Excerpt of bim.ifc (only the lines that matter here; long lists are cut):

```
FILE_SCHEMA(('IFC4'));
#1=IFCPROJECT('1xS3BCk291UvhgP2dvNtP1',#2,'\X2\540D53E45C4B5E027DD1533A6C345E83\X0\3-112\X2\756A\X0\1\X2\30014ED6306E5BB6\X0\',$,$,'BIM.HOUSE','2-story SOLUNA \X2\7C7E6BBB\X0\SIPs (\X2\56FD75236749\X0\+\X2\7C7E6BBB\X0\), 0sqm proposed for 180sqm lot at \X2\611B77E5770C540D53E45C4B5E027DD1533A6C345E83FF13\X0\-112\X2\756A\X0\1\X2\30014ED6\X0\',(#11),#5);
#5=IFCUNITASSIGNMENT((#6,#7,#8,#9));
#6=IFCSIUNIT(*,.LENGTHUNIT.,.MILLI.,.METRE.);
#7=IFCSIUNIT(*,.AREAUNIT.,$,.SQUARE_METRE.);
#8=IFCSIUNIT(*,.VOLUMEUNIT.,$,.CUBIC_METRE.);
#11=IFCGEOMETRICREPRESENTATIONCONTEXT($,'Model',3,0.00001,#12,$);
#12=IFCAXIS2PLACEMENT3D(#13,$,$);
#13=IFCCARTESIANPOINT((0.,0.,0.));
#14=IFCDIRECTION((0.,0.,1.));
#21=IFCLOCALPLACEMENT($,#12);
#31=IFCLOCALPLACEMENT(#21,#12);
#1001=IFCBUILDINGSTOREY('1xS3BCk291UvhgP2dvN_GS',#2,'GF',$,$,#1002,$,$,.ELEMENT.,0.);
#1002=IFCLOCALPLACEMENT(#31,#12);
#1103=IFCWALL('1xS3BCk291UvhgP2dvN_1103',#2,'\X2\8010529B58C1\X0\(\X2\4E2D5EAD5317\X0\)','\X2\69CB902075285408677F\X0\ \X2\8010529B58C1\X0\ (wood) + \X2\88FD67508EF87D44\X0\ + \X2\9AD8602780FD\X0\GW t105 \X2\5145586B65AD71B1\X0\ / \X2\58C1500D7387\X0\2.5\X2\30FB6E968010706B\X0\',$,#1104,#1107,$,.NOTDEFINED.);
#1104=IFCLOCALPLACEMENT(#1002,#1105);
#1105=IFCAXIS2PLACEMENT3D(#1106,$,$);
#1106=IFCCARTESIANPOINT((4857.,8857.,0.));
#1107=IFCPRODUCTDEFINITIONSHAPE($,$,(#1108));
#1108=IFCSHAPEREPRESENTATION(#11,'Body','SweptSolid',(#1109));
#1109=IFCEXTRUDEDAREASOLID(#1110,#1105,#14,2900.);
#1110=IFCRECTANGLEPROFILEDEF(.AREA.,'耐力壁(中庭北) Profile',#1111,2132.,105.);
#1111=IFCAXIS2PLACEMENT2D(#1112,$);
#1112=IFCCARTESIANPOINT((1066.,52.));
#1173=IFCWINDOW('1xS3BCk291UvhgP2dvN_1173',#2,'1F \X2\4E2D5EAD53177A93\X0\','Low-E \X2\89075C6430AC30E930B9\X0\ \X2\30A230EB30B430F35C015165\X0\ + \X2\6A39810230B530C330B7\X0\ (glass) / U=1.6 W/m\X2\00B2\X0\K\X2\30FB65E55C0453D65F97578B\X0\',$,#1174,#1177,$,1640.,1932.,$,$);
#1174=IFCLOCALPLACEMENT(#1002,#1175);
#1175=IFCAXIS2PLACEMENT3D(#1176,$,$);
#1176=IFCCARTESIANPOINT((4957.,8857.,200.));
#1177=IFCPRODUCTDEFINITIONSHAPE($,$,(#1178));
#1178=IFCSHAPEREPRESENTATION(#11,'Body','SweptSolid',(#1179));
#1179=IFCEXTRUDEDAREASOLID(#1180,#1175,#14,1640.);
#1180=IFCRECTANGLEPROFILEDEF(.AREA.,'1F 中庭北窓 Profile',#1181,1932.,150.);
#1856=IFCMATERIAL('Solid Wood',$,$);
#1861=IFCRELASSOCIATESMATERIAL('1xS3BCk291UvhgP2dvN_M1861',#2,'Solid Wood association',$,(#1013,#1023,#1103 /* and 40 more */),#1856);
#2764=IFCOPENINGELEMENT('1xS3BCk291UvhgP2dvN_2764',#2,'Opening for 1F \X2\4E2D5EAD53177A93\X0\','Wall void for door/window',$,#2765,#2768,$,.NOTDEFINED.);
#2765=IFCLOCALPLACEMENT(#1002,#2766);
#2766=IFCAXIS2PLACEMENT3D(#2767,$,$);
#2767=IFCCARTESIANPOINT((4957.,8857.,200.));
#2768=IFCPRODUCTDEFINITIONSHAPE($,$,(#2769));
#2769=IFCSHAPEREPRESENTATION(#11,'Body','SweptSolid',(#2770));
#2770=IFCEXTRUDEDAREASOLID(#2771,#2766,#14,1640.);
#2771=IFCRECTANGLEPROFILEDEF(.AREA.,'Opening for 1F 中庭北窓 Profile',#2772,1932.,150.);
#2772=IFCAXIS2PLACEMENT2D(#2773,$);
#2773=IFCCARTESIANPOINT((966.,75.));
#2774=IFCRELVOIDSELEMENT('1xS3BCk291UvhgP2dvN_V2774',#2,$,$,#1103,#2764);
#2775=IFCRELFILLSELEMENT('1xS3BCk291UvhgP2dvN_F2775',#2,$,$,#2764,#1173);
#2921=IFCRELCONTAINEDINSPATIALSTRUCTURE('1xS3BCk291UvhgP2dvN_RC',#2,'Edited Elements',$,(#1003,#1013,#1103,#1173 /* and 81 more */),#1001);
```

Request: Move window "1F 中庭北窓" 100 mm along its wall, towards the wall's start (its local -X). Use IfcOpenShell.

```python
import ifcopenshell
import ifcopenshell.api.geometry
import ifcopenshell.util.placement
import ifcopenshell.util.unit

model = ifcopenshell.open("bim.ifc")
unit_scale = ifcopenshell.util.unit.calculate_unit_scale(model)

window = model.by_guid("1xS3BCk291UvhgP2dvN_1173")
opening = window.FillsVoids[0].RelatingOpeningElement
wall = opening.VoidsElements[0].RelatingBuildingElement

wall_matrix = ifcopenshell.util.placement.get_local_placement(wall.ObjectPlacement)
shift = wall_matrix[:3, 0] * -0.1 / unit_scale
before = ifcopenshell.util.placement.get_local_placement(window.ObjectPlacement)[:3, 3].copy()

# The window is not placed relative to its opening, so move both.
for product in (opening, window):
    matrix = ifcopenshell.util.placement.get_local_placement(product.ObjectPlacement)
    matrix[:3, 3] += shift
    ifcopenshell.api.geometry.edit_object_placement(model, product=product, matrix=matrix, is_si=False)

after = ifcopenshell.util.placement.get_local_placement(window.ObjectPlacement)[:3, 3]
print("window moved by", (after - before).round(3) + 0.0)

model.write("bim_edited.ifc")
```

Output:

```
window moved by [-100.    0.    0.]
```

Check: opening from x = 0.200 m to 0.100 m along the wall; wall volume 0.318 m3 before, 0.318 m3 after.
